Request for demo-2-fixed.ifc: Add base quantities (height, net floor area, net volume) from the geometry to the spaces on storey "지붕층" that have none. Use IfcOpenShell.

First a look at what the model holds.

```python
import ifcopenshell
import ifcopenshell.util.element
import ifcopenshell.util.unit

model = ifcopenshell.open("demo-2-fixed.ifc")
print(model.schema)
for unit_type in ("LENGTHUNIT", "AREAUNIT", "VOLUMEUNIT"):
    print(unit_type, ifcopenshell.util.unit.calculate_unit_scale(model, unit_type))
storey = next(s for s in model.by_type("IfcBuildingStorey") if s.Name == "지붕층")
spaces = [e for e in ifcopenshell.util.element.get_decomposition(storey) if e.is_a("IfcSpace")]
for e in sorted(spaces, key=lambda e: e.id()):
    print(e.id(), e.is_a(), e.Name, list(ifcopenshell.util.element.get_psets(e, qtos_only=True)), sep=" | ")
```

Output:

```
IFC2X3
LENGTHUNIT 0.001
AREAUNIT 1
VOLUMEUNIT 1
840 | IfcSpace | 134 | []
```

```python
import ifcopenshell
import ifcopenshell.api.pset
import ifcopenshell.geom
import ifcopenshell.util.element
import ifcopenshell.util.shape
import ifcopenshell.util.unit

model = ifcopenshell.open("demo-2-fixed.ifc")
unit_scale = ifcopenshell.util.unit.calculate_unit_scale(model)
area_scale = ifcopenshell.util.unit.calculate_unit_scale(model, "AREAUNIT")
volume_scale = ifcopenshell.util.unit.calculate_unit_scale(model, "VOLUMEUNIT")
settings = ifcopenshell.geom.settings()

storey = next(s for s in model.by_type("IfcBuildingStorey") if s.Name == "지붕층")
spaces = [e for e in ifcopenshell.util.element.get_decomposition(storey) if e.is_a("IfcSpace")]

for e in sorted(spaces, key=lambda e: e.id()):
    if ifcopenshell.util.element.get_psets(e, qtos_only=True, should_inherit=False):
        continue
    # Geometry comes back in metres, in the element's own axes.
    shape = ifcopenshell.geom.create_shape(settings, e)
    values = {
        "Height": ifcopenshell.util.shape.get_z(shape.geometry) / unit_scale,
        "NetFloorArea": ifcopenshell.util.shape.get_footprint_area(shape.geometry) / area_scale,
        "NetVolume": ifcopenshell.util.shape.get_volume(shape.geometry) / volume_scale,
    }
    qto = ifcopenshell.api.pset.add_qto(model, product=e, name="BaseQuantities")
    ifcopenshell.api.pset.edit_qto(model, qto=qto, properties=values)
    print(e.id(), {k: round(v, 3) for k, v in values.items()})

model.write("demo-2-fixed_rev.ifc")
```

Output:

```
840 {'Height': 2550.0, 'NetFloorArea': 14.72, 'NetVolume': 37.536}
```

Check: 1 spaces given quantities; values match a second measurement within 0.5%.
